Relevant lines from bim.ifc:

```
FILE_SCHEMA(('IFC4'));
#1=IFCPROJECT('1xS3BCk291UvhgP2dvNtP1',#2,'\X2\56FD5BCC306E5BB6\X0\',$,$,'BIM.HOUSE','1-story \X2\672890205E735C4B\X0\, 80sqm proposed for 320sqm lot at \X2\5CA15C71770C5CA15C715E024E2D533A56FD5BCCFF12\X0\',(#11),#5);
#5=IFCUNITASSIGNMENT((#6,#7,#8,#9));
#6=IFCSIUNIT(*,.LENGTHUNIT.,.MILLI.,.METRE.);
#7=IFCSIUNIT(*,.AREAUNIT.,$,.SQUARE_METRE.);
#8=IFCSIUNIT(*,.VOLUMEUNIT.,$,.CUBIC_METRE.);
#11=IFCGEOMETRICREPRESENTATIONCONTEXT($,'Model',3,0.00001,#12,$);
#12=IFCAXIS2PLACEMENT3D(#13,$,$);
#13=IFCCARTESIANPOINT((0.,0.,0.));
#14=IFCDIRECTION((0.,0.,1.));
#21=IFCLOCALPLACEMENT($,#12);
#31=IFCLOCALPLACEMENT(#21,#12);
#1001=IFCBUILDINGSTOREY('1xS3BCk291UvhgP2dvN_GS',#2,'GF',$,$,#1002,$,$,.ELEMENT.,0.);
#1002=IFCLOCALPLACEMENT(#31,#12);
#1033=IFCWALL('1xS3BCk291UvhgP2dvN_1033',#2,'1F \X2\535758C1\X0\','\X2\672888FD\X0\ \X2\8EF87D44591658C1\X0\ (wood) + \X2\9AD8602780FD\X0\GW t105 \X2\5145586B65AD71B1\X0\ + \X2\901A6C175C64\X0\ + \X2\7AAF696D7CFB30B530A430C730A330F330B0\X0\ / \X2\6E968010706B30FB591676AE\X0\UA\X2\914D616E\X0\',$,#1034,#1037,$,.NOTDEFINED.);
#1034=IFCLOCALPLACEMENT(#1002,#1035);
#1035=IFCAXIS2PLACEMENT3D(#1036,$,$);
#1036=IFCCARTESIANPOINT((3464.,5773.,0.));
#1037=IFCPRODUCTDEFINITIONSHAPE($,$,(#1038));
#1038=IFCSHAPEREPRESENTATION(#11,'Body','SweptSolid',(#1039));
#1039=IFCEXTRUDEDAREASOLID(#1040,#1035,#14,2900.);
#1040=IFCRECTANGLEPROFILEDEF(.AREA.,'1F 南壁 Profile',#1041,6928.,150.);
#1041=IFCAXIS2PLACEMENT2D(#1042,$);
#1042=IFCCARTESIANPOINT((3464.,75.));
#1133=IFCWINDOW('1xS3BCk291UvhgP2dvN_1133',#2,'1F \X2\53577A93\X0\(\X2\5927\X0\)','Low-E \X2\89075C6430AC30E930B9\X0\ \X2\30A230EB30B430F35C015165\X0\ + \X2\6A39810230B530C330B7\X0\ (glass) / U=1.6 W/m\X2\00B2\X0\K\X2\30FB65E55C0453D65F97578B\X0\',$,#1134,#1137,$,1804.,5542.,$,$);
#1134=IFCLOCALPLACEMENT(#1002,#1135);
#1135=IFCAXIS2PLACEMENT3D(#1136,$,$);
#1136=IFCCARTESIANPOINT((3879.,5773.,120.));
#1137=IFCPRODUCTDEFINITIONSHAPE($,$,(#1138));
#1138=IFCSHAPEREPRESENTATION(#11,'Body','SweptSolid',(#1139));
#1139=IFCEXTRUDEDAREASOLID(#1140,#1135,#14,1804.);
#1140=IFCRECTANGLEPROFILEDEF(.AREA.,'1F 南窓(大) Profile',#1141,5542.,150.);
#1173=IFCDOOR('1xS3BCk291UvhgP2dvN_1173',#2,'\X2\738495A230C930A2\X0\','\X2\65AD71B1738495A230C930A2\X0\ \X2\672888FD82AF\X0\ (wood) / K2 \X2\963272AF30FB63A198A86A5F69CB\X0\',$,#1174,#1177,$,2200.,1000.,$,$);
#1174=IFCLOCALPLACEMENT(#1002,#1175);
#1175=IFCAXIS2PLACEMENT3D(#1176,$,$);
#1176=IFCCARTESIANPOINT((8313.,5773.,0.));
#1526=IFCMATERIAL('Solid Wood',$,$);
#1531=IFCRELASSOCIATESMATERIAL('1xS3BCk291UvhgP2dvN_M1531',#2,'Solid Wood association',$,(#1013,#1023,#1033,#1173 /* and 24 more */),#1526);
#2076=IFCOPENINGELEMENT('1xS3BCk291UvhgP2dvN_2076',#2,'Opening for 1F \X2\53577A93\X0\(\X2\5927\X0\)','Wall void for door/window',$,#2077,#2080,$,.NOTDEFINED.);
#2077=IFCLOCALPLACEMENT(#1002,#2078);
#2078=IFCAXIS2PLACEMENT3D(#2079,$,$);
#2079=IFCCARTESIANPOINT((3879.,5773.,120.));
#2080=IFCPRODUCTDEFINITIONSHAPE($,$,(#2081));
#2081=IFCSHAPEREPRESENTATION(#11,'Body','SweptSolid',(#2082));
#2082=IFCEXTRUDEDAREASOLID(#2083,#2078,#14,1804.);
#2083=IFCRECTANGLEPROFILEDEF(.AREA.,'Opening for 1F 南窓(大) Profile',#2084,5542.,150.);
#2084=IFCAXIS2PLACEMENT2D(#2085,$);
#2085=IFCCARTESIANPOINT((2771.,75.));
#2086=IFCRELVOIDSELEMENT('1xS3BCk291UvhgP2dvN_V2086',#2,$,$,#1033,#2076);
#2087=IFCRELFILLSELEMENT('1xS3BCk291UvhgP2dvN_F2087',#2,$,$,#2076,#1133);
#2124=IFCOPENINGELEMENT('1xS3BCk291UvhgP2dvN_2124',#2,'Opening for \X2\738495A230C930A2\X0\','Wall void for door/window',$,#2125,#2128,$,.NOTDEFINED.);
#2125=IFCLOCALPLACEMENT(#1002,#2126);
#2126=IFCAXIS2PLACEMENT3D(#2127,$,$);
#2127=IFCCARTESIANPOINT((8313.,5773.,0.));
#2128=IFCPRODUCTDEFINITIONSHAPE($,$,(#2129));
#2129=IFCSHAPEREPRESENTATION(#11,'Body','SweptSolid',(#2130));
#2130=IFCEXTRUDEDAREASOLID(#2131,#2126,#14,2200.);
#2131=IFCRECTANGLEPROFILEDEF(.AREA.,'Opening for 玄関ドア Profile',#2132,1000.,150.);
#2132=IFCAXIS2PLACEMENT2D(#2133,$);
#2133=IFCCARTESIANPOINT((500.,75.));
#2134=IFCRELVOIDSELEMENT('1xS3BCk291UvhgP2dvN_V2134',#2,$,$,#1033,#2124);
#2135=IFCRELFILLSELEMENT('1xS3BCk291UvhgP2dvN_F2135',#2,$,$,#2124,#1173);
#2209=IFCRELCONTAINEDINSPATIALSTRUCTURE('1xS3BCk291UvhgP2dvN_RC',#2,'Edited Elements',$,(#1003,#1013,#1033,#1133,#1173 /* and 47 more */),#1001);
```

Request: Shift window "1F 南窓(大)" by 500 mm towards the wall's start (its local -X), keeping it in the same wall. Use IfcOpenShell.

```python
import ifcopenshell
import ifcopenshell.api.geometry
import ifcopenshell.util.placement
import ifcopenshell.util.unit

model = ifcopenshell.open("bim.ifc")
unit_scale = ifcopenshell.util.unit.calculate_unit_scale(model)

window = model.by_id(1133)
opening = window.FillsVoids[0].RelatingOpeningElement
wall = opening.VoidsElements[0].RelatingBuildingElement

wall_matrix = ifcopenshell.util.placement.get_local_placement(wall.ObjectPlacement)
shift = wall_matrix[:3, 0] * -0.5 / unit_scale
before = ifcopenshell.util.placement.get_local_placement(window.ObjectPlacement)[:3, 3].copy()

# The window is not placed relative to its opening, so move both.
for product in (opening, window):
    matrix = ifcopenshell.util.placement.get_local_placement(product.ObjectPlacement)
    matrix[:3, 3] += shift
    ifcopenshell.api.geometry.edit_object_placement(model, product=product, matrix=matrix, is_si=False)

after = ifcopenshell.util.placement.get_local_placement(window.ObjectPlacement)[:3, 3]
print("window moved by", (after - before).round(3) + 0.0)

model.write("bim-out.ifc")
```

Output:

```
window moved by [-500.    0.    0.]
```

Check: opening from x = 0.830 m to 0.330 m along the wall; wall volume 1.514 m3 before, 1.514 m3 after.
